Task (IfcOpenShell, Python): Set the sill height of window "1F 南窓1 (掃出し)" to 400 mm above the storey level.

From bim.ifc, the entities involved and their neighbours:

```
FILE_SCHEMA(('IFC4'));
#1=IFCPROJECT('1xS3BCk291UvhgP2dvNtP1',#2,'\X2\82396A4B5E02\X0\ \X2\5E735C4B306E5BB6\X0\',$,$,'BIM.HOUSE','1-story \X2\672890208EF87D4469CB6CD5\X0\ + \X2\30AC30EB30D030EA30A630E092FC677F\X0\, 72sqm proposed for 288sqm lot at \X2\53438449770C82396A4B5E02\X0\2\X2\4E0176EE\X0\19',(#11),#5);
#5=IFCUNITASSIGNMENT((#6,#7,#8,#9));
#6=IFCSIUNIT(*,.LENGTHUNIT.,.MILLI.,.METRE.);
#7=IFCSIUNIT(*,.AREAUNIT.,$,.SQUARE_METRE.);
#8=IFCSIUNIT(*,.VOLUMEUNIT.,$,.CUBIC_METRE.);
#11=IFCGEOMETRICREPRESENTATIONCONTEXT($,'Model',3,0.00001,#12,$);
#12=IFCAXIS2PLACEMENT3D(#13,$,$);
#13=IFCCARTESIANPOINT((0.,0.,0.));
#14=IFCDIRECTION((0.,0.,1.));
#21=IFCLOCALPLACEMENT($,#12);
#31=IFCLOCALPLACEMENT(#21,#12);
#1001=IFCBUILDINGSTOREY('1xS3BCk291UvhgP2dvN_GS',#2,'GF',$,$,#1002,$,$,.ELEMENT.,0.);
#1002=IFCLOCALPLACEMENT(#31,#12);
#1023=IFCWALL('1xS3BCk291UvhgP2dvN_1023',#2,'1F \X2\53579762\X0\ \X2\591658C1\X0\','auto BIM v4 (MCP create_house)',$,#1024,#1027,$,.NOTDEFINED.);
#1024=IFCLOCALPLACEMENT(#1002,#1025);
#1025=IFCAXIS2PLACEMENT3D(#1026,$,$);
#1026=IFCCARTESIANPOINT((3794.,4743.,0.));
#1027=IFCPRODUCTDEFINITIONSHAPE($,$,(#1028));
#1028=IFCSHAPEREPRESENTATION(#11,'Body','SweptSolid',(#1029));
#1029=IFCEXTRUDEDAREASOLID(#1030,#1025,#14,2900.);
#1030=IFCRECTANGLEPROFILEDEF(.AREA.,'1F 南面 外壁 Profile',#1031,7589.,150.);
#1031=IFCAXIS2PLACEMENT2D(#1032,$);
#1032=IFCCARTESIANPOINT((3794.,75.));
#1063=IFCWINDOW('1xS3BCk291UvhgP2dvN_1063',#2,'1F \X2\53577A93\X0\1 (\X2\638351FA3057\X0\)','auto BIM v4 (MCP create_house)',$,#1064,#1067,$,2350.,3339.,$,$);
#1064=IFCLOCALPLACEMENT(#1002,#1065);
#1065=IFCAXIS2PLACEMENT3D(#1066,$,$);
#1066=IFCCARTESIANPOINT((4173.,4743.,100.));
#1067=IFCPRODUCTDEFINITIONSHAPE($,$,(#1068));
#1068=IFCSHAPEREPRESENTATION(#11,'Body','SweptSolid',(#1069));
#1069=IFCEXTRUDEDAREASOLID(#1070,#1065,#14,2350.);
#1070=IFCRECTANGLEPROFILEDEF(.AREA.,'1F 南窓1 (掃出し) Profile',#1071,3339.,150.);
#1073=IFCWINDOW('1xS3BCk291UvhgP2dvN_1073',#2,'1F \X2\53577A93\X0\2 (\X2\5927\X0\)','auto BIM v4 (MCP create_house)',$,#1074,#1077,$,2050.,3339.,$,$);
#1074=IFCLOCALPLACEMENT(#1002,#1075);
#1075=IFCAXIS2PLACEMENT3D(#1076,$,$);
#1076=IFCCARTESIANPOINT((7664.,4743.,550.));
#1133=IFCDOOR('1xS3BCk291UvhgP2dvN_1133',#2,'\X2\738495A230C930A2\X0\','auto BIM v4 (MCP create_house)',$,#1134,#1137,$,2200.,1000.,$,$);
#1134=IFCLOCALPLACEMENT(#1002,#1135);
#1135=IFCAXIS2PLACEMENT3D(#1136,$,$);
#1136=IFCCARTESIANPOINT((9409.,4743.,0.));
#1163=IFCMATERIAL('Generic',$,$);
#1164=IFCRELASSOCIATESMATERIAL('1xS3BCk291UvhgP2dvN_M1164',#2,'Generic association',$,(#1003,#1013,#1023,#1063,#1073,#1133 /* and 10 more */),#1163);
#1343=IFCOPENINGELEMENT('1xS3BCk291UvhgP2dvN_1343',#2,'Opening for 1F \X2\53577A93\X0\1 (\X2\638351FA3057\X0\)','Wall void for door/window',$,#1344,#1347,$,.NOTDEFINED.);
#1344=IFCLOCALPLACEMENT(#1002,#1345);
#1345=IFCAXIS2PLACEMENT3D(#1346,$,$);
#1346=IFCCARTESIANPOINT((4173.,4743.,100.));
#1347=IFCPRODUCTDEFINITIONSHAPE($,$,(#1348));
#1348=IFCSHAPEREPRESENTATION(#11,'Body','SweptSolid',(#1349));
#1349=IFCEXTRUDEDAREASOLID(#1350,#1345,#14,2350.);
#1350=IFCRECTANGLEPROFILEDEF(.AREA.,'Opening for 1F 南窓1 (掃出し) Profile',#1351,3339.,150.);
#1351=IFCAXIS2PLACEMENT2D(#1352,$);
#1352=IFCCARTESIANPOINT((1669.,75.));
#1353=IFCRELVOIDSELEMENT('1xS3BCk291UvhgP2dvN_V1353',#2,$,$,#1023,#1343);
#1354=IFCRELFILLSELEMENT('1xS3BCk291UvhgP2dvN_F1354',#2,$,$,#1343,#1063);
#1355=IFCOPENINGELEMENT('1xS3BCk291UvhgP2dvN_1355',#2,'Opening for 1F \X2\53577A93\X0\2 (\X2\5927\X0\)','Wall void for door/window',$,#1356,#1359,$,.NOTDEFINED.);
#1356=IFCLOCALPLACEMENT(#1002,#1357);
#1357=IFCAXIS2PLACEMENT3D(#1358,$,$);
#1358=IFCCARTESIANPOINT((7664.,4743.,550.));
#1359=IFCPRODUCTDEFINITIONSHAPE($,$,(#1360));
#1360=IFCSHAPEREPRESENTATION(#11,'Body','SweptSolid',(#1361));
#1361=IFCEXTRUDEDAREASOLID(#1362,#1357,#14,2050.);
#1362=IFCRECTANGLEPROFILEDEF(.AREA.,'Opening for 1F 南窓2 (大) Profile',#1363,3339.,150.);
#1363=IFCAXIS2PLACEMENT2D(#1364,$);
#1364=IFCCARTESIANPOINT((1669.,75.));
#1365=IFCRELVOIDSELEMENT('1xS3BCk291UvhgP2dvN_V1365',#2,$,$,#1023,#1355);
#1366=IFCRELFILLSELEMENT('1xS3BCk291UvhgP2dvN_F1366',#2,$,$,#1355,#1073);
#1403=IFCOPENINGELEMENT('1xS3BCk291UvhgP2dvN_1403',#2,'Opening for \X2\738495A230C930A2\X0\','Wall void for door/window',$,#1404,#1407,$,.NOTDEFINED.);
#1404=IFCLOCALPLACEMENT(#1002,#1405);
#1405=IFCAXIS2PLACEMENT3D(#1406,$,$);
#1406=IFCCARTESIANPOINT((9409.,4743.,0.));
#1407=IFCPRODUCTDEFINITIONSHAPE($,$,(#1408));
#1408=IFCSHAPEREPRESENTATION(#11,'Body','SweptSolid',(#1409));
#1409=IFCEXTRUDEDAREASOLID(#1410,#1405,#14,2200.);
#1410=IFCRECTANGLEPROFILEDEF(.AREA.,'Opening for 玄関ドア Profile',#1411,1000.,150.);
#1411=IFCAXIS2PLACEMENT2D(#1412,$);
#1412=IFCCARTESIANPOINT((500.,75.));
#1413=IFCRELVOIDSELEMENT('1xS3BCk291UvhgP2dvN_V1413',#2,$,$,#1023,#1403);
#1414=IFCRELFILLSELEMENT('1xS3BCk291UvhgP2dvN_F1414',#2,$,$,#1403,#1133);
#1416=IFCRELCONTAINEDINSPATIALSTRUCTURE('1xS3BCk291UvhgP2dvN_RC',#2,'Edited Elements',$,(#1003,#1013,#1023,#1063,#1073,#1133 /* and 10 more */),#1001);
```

```python
import numpy as np
import ifcopenshell
import ifcopenshell.api.geometry
import ifcopenshell.geom
import ifcopenshell.util.element
import ifcopenshell.util.placement
import ifcopenshell.util.shape
import ifcopenshell.util.unit

model = ifcopenshell.open("bim.ifc")
unit_scale = ifcopenshell.util.unit.calculate_unit_scale(model)

window = model.by_guid("1xS3BCk291UvhgP2dvN_1063")
opening = window.FillsVoids[0].RelatingOpeningElement
storey = ifcopenshell.util.element.get_container(window, ifc_class="IfcBuildingStorey")
level = ifcopenshell.util.placement.get_local_placement(storey.ObjectPlacement)[2, 3]

# The opening's origin need not be at the sill, so measure its lowest point.
shape = ifcopenshell.geom.create_shape(ifcopenshell.geom.settings(), opening)
bottom = ifcopenshell.util.shape.get_shape_bottom_elevation(shape, shape.geometry) / unit_scale
dz = level + 400.0 - bottom

shift = np.array([0.0, 0.0, dz])
# The window is not placed relative to its opening, so move both.
for product in (opening, window):
    matrix = ifcopenshell.util.placement.get_local_placement(product.ObjectPlacement)
    matrix[:3, 3] += shift
    ifcopenshell.api.geometry.edit_object_placement(model, product=product, matrix=matrix, is_si=False)

print(f"moved by {dz * unit_scale:+.3f} m")

model.write("bim_v2.ifc")
```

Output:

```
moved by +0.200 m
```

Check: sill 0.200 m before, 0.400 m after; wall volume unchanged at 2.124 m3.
